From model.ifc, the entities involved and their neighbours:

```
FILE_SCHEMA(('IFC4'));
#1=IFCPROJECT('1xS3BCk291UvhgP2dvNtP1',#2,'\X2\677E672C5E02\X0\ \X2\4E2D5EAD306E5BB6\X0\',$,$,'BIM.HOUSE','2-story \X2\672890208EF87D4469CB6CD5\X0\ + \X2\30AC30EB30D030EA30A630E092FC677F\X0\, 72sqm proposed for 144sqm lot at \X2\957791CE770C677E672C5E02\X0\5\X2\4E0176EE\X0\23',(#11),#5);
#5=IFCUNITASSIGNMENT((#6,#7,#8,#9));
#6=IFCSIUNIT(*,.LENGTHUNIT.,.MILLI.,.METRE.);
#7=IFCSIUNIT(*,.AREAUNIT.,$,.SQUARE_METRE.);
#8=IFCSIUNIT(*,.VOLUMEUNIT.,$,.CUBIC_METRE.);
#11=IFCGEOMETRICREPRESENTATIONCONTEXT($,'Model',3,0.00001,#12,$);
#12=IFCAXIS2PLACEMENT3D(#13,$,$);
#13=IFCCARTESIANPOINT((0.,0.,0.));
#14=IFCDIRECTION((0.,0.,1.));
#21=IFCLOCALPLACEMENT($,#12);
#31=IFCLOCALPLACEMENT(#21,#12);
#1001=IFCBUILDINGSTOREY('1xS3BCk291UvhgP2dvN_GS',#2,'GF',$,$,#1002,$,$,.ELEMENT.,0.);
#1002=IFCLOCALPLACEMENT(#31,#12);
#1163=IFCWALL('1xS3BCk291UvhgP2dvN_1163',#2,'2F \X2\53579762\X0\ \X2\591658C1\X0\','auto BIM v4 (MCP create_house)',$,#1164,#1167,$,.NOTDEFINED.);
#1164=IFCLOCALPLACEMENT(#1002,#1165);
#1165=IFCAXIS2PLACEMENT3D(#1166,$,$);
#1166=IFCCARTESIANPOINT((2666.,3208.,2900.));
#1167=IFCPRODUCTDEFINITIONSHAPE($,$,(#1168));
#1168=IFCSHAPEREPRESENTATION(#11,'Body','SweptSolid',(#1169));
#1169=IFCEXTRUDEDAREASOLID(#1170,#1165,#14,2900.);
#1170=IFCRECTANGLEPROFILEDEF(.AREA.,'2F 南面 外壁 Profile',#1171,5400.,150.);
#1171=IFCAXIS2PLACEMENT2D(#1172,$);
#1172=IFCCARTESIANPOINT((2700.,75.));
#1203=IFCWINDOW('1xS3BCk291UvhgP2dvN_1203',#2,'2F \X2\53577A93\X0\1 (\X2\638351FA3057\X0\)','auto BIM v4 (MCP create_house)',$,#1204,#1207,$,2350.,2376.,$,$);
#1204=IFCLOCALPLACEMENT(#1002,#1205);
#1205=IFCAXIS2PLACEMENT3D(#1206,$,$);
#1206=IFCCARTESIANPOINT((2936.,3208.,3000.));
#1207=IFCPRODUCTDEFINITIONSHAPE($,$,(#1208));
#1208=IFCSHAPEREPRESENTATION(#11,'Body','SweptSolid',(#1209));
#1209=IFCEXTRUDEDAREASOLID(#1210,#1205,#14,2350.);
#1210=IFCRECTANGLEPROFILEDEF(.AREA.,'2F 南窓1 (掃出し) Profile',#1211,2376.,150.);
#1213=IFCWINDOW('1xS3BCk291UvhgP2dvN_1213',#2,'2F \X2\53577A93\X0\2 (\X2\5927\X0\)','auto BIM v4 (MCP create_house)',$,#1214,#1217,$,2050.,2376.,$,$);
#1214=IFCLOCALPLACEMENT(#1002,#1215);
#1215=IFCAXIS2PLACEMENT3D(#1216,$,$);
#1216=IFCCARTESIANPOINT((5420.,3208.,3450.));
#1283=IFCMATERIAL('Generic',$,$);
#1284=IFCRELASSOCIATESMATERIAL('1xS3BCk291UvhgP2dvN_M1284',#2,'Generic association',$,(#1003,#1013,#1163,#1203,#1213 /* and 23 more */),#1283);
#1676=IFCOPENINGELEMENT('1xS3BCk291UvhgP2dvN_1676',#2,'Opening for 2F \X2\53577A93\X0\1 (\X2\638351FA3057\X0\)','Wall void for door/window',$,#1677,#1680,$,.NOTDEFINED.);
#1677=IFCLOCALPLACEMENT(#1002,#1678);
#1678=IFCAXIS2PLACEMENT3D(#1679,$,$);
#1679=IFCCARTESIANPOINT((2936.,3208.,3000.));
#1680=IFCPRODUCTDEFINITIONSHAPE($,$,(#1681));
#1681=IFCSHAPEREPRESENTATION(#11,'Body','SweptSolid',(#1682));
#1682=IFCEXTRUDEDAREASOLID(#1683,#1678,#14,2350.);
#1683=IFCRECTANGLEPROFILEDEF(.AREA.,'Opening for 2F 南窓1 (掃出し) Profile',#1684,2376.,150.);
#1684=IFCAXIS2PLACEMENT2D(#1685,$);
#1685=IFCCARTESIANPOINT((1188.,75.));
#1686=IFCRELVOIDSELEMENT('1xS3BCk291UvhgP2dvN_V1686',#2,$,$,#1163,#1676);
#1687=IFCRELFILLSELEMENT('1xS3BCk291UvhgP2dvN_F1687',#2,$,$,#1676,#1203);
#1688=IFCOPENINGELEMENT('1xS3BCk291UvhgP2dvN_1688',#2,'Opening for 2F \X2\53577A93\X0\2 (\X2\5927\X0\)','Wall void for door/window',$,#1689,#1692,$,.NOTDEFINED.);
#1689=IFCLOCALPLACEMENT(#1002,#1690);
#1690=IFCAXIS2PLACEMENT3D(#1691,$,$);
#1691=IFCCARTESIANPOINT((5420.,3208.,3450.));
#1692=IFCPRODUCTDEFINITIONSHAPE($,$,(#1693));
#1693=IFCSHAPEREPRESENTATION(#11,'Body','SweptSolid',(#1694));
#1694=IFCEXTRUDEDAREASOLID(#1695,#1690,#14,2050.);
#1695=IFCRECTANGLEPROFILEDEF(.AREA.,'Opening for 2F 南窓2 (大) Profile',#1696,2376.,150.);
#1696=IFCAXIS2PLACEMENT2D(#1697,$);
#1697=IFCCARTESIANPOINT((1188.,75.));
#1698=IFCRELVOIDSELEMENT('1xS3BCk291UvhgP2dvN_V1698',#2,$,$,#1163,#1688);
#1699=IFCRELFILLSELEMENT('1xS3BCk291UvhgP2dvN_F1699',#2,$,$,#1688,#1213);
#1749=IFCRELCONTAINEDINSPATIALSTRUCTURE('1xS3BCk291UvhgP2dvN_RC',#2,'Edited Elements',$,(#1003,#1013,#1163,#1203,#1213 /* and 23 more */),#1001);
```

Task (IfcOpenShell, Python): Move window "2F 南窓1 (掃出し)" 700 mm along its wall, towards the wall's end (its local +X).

```python
import ifcopenshell
import ifcopenshell.api.geometry
import ifcopenshell.util.placement
import ifcopenshell.util.unit

model = ifcopenshell.open("model.ifc")
unit_scale = ifcopenshell.util.unit.calculate_unit_scale(model)

window = model.by_id(1203)
opening = window.FillsVoids[0].RelatingOpeningElement
wall = opening.VoidsElements[0].RelatingBuildingElement

wall_matrix = ifcopenshell.util.placement.get_local_placement(wall.ObjectPlacement)
shift = wall_matrix[:3, 0] * 0.7 / unit_scale
before = ifcopenshell.util.placement.get_local_placement(window.ObjectPlacement)[:3, 3].copy()

# The window is not placed relative to its opening, so move both.
for product in (opening, window):
    matrix = ifcopenshell.util.placement.get_local_placement(product.ObjectPlacement)
    matrix[:3, 3] += shift
    ifcopenshell.api.geometry.edit_object_placement(model, product=product, matrix=matrix, is_si=False)

after = ifcopenshell.util.placement.get_local_placement(window.ObjectPlacement)[:3, 3]
print("window moved by", (after - before).round(3) + 0.0)

model.write("model-out.ifc")
```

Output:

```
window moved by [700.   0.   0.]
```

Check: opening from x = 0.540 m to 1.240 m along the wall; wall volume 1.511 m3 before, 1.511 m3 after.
